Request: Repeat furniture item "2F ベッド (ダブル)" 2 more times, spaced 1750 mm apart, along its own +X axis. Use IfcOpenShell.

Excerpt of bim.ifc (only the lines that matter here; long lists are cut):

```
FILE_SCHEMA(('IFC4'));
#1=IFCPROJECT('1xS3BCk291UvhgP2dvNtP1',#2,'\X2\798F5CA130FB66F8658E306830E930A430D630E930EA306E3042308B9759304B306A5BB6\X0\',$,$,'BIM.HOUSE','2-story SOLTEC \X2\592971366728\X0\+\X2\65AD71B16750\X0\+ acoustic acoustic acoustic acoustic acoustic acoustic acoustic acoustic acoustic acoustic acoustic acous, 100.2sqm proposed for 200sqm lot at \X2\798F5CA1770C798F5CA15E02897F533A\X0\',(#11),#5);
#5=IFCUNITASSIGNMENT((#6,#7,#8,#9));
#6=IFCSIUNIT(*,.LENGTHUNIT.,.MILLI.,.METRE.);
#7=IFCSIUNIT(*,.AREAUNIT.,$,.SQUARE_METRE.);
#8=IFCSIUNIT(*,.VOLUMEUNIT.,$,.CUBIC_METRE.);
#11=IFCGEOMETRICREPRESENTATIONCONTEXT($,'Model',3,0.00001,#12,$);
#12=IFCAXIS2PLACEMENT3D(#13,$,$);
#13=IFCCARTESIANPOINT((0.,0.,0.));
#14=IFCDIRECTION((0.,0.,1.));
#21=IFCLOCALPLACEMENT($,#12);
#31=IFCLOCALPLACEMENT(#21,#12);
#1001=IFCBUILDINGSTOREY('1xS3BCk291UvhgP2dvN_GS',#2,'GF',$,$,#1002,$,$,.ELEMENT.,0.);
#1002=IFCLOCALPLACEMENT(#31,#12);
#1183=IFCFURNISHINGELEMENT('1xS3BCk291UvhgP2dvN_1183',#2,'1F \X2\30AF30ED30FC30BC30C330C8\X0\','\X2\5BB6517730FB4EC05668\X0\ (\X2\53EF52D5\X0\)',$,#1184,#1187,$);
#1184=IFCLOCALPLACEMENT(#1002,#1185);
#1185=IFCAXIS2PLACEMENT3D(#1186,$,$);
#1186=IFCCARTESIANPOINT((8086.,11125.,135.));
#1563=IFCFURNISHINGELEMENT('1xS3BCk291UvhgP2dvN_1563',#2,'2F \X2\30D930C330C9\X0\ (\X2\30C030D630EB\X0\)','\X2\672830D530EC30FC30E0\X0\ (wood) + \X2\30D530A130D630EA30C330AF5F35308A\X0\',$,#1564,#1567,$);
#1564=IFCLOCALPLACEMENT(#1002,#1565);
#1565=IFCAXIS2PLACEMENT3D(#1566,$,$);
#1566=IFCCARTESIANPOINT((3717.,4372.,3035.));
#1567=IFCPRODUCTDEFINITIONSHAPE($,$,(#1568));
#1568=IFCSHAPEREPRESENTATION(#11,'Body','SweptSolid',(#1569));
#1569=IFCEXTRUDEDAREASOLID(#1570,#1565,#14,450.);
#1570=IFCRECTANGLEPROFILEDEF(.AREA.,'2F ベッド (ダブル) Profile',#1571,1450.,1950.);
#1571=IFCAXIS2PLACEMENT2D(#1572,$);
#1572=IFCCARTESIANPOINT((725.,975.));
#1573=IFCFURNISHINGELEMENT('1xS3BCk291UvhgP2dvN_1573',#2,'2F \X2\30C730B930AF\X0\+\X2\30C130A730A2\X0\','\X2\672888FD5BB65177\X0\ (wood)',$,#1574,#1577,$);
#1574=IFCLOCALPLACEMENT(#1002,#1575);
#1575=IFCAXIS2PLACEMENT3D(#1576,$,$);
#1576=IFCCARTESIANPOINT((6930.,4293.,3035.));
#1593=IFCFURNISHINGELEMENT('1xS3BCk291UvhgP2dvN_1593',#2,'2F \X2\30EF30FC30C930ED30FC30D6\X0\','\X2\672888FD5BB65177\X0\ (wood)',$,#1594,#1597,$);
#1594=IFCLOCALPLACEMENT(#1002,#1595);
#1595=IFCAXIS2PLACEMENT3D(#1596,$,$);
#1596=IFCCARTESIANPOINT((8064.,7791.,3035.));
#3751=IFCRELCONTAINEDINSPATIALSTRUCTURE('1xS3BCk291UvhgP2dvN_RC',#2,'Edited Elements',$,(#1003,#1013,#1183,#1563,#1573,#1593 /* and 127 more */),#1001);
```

```python
import ifcopenshell
import ifcopenshell.api.geometry
import ifcopenshell.api.root
import ifcopenshell.util.element
import ifcopenshell.util.placement

model = ifcopenshell.open("bim.ifc")


def reuse_history(source, copy):
    """copy_class also copies each property set's owner history, people and application; keep the originals."""
    for rel in copy.IsDefinedBy:
        if rel.is_a("IfcRelDefinesByProperties") and (history := rel.RelatingPropertyDefinition.OwnerHistory):
            rel.RelatingPropertyDefinition.OwnerHistory = source.OwnerHistory
            ifcopenshell.util.element.remove_deep2(model, history)


source = model.by_guid("1xS3BCk291UvhgP2dvN_1563")
base = ifcopenshell.util.placement.get_local_placement(source.ObjectPlacement)
step = base[:3, 0] * 1750.0

for i in range(1, 3):
    copy = ifcopenshell.api.root.copy_class(model, product=source)
    copy.Representation = ifcopenshell.util.element.copy_deep(
        model, source.Representation, exclude=["IfcGeometricRepresentationContext", "IfcRepresentationMap"]
    )
    reuse_history(source, copy)
    matrix = base.copy()
    matrix[:3, 3] += i * step
    print("added at", matrix[:3, 3].round(3) + 0.0)
    ifcopenshell.api.geometry.edit_object_placement(model, product=copy, matrix=matrix, is_si=False)

model.write("bim_updated.ifc")
```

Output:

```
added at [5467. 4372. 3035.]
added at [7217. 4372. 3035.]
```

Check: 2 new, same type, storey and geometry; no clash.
